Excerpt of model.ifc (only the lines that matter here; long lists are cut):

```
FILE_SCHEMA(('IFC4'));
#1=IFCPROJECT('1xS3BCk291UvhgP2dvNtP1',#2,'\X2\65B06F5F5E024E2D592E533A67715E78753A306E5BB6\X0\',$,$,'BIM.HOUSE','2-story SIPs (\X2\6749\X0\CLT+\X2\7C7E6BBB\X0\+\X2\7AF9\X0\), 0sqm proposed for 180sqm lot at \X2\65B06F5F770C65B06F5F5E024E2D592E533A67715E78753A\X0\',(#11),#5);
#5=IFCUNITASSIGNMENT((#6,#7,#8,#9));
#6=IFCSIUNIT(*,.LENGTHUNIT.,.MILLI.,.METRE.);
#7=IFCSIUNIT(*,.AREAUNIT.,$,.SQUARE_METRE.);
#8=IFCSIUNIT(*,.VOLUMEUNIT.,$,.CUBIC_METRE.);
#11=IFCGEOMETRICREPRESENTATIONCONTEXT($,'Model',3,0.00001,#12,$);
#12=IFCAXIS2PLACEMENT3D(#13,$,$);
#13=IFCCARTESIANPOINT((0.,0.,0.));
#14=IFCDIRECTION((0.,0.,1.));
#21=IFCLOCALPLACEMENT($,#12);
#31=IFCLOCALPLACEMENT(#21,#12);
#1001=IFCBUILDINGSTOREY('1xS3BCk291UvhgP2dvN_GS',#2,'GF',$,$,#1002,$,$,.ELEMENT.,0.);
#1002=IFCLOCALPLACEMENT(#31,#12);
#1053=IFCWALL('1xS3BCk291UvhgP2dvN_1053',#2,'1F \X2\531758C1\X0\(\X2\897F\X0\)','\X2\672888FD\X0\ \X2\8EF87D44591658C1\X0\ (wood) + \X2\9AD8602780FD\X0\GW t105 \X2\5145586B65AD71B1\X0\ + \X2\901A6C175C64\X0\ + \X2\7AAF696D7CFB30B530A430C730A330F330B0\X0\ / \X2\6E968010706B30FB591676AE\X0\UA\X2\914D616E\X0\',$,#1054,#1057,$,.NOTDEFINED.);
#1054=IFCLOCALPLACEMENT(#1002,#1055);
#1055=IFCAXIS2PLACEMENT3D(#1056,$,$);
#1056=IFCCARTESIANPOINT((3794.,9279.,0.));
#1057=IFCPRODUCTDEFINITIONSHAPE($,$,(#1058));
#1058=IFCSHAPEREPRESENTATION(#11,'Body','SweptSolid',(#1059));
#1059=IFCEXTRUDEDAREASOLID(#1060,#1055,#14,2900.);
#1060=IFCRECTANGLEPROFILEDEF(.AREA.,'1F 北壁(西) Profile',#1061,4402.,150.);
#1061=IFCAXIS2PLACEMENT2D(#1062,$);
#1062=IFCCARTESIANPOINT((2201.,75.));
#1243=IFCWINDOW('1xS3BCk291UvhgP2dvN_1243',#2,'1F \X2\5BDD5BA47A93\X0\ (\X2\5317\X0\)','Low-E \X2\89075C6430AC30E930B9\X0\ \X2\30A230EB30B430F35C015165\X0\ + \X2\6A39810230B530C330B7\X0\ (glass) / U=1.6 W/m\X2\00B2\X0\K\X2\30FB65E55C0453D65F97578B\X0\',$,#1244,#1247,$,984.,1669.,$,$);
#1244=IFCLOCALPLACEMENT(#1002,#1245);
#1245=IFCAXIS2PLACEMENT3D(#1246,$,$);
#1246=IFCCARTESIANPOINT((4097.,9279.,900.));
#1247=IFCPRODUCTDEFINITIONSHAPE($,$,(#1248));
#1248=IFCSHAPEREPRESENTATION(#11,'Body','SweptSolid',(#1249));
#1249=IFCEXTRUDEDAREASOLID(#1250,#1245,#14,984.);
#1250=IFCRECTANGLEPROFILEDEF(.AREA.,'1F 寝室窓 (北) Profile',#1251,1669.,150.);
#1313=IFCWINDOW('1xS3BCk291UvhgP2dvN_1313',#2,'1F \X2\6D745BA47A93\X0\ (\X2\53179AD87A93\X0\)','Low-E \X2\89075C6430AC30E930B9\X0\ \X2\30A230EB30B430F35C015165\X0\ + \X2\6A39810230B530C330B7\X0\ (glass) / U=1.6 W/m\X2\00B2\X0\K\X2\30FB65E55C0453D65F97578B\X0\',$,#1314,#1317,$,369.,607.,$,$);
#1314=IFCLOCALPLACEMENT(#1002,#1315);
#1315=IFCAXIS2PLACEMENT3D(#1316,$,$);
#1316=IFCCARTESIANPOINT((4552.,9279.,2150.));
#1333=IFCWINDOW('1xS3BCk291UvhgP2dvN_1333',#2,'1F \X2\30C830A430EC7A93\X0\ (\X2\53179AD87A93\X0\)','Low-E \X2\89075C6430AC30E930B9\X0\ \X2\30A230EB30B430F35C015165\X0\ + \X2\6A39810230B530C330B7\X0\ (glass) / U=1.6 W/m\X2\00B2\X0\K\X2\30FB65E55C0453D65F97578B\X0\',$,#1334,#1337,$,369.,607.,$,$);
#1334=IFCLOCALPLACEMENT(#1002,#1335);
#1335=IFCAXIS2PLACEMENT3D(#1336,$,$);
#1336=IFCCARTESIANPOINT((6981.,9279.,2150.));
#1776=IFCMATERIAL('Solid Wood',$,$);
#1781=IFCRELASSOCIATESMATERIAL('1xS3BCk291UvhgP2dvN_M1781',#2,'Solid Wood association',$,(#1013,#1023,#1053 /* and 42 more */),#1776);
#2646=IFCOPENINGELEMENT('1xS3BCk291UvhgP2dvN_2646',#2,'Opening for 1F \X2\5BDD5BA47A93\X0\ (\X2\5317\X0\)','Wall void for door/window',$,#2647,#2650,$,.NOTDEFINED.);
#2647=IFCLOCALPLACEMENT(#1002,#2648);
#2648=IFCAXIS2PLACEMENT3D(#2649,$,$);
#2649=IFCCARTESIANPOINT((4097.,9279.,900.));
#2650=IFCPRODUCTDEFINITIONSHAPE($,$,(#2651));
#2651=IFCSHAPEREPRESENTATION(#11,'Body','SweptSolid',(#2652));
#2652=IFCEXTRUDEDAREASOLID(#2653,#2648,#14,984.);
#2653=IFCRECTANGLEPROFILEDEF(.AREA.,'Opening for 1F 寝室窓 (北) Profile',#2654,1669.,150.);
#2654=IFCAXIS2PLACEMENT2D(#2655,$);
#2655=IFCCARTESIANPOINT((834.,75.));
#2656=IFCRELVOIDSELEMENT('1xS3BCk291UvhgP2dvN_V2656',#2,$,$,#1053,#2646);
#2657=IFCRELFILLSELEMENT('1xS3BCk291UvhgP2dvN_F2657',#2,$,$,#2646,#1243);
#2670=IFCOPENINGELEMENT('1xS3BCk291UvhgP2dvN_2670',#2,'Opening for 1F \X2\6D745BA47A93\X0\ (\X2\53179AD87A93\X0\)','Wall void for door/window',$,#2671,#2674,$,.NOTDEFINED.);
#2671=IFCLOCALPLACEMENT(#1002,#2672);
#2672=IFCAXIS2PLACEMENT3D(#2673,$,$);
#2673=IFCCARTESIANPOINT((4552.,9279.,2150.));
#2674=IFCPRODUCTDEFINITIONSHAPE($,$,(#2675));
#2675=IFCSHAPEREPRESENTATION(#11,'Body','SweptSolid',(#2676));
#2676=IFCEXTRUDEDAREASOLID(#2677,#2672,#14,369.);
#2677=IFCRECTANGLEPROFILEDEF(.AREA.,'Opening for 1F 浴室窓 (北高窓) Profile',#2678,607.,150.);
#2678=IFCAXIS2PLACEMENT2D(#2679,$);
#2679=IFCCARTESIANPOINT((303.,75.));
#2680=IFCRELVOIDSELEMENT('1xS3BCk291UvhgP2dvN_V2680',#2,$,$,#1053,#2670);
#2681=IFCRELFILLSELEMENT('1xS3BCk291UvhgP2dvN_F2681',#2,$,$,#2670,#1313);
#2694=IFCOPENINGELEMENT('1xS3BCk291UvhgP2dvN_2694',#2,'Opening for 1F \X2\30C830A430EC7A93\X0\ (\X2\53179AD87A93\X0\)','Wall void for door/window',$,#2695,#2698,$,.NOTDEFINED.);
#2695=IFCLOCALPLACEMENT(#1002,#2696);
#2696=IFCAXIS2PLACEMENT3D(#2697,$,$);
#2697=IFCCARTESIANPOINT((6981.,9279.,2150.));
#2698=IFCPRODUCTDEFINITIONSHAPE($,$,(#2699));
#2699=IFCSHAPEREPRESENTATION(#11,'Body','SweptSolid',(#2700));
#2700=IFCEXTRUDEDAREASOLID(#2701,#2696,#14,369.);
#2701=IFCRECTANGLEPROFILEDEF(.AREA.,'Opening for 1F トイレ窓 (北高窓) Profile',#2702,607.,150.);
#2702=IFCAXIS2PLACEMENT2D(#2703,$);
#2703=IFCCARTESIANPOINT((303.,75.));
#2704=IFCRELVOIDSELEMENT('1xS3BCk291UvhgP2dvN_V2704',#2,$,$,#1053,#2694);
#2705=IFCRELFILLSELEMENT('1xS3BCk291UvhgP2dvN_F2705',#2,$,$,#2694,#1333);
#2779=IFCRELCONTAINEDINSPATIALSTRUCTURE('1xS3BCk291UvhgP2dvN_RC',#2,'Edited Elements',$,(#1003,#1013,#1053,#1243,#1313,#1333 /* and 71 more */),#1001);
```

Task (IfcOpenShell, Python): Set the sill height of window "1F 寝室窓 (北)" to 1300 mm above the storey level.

```python
import numpy as np
import ifcopenshell
import ifcopenshell.api.geometry
import ifcopenshell.geom
import ifcopenshell.util.element
import ifcopenshell.util.placement
import ifcopenshell.util.shape
import ifcopenshell.util.unit

model = ifcopenshell.open("model.ifc")
unit_scale = ifcopenshell.util.unit.calculate_unit_scale(model)

window = model.by_guid("1xS3BCk291UvhgP2dvN_1243")
opening = window.FillsVoids[0].RelatingOpeningElement
storey = ifcopenshell.util.element.get_container(window, ifc_class="IfcBuildingStorey")
level = ifcopenshell.util.placement.get_local_placement(storey.ObjectPlacement)[2, 3]

# The opening's origin need not be at the sill, so measure its lowest point.
shape = ifcopenshell.geom.create_shape(ifcopenshell.geom.settings(), opening)
bottom = ifcopenshell.util.shape.get_shape_bottom_elevation(shape, shape.geometry) / unit_scale
dz = level + 1.3 / unit_scale - bottom

shift = np.array([0.0, 0.0, dz])
# The window is not placed relative to its opening, so move both.
for product in (opening, window):
    matrix = ifcopenshell.util.placement.get_local_placement(product.ObjectPlacement)
    matrix[:3, 3] += shift
    ifcopenshell.api.geometry.edit_object_placement(model, product=product, matrix=matrix, is_si=False)

print(f"moved by {dz * unit_scale:+.3f} m")

model.write("model_updated.ifc")
```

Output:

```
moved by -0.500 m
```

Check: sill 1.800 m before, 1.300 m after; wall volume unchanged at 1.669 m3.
